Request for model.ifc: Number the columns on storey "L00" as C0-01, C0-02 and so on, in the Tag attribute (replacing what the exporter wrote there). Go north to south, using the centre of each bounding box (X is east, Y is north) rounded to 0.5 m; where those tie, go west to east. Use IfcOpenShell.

First a look at what the model holds.

```python
import ifcopenshell
import ifcopenshell.util.element
import ifcopenshell.util.placement

model = ifcopenshell.open("model.ifc")
print(model.schema)
storey = next(s for s in model.by_type("IfcBuildingStorey") if s.Name == "L00")
columns = [e for e in ifcopenshell.util.element.get_decomposition(storey) if e.is_a("IfcColumn")]
for e in sorted(columns, key=lambda e: e.id()):
    origin = ifcopenshell.util.placement.get_local_placement(e.ObjectPlacement)[:3, 3]
    print(e.id(), e.Tag, e.Name, origin.round(2) + 0.0, sep=" | ")
```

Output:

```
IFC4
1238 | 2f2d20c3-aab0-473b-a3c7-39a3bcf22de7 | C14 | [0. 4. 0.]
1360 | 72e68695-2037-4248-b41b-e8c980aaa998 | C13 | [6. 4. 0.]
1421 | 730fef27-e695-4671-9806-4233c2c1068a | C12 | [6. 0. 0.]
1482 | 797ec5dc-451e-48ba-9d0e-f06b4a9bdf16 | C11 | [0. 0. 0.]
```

```python
import ifcopenshell
import ifcopenshell.geom
import ifcopenshell.util.element
import ifcopenshell.util.shape

model = ifcopenshell.open("model.ifc")
settings = ifcopenshell.geom.settings()
settings.set("use-world-coords", True)


def centre(element):
    shape = ifcopenshell.geom.create_shape(settings, element)
    return ifcopenshell.util.shape.get_bbox_centroid(shape.geometry)


storey = next(s for s in model.by_type("IfcBuildingStorey") if s.Name == "L00")
columns = [e for e in ifcopenshell.util.element.get_decomposition(storey) if e.is_a("IfcColumn")]

# Insertion points can sit at a corner or the storey origin, so sort by the geometry (in metres).
centres = {e: centre(e) for e in columns}
columns.sort(key=lambda e: (-round(centres[e][1] / 0.5), centres[e][0]))

for i, e in enumerate(columns, start=1):
    number = f"C0-{i:02d}"
    e.Tag = number
    print(e.id(), number)

model.write("model_updated.ifc")
```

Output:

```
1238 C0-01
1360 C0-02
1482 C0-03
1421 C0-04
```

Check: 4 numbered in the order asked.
